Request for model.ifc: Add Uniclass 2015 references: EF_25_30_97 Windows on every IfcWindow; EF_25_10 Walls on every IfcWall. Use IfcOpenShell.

First a look at what the model holds.

```python
import ifcopenshell

model = ifcopenshell.open("model.ifc")
print(model.schema)
print("classifications:", [c.Name for c in model.by_type("IfcClassification")])
for ifc_class in ("IfcDoor", "IfcRoof", "IfcStair", "IfcWall", "IfcWindow"):
    print(ifc_class, len(model.by_type(ifc_class)))
```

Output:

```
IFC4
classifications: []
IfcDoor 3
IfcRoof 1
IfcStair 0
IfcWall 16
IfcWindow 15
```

```python
import ifcopenshell
import ifcopenshell.api.classification

model = ifcopenshell.open("model.ifc")

system = ifcopenshell.api.classification.add_classification(model, classification="Uniclass 2015")

codes = {
    "IfcWindow": ("EF_25_30_97", "Windows"),
    "IfcWall": ("EF_25_10", "Walls"),
}
for ifc_class, (code, name) in codes.items():
    products = model.by_type(ifc_class)
    ifcopenshell.api.classification.add_reference(
        model, products=products, classification=system, identification=code, name=name
    )
    print(code, len(products))

model.write("model_updated.ifc")
```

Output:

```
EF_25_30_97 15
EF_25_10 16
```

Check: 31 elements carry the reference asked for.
